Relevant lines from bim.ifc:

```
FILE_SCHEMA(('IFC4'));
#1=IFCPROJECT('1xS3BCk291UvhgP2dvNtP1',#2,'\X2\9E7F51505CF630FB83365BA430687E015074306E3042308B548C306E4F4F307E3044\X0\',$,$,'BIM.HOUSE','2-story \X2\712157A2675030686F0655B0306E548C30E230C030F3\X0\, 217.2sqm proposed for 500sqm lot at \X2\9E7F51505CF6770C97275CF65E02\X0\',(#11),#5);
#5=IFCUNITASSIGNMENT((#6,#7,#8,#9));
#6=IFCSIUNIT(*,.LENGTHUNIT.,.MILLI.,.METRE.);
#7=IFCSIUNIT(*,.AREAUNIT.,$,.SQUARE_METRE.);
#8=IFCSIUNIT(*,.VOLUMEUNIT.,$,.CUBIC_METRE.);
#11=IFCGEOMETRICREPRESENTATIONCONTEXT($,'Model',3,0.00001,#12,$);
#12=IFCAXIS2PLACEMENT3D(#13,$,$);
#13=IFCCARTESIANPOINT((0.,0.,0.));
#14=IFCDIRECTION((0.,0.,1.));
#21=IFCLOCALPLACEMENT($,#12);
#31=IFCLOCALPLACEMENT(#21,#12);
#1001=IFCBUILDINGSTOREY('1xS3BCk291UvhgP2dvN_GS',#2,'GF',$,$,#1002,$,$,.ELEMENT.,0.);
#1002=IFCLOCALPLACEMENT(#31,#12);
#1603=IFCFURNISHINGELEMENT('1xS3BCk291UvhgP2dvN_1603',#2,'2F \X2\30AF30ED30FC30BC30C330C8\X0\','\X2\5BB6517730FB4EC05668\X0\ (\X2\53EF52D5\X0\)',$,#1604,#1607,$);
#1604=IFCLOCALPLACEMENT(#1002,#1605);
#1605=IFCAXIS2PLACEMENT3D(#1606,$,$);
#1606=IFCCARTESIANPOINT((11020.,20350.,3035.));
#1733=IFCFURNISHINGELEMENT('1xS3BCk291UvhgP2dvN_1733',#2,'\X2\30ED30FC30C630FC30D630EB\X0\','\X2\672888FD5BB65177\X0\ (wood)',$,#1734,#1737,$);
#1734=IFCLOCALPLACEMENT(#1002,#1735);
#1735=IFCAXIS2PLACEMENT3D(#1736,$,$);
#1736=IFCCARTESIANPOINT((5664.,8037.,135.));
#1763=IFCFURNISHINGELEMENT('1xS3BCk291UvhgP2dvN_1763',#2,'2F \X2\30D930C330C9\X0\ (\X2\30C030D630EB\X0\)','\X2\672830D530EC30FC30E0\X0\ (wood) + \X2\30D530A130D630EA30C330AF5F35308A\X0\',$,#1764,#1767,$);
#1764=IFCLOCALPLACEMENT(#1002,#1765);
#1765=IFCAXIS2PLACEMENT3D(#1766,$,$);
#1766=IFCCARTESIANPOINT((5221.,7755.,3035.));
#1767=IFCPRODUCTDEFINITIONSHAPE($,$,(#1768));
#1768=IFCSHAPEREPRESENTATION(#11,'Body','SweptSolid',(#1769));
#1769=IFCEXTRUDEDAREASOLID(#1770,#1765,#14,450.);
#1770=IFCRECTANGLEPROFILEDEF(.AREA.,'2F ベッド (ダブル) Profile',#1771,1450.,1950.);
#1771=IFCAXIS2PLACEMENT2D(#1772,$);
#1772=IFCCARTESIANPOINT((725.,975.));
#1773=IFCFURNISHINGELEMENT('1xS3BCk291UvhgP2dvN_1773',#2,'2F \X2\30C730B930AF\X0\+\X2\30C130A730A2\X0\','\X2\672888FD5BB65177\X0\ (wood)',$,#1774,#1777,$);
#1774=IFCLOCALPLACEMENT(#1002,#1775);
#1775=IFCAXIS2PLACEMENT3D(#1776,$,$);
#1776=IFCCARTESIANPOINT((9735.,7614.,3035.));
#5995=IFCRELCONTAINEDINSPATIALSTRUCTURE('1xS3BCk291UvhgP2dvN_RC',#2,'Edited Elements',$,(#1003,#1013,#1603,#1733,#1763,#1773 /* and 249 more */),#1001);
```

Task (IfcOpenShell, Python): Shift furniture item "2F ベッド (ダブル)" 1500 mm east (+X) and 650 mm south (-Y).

```python
import ifcopenshell
import ifcopenshell.api.geometry
import ifcopenshell.util.placement

model = ifcopenshell.open("bim.ifc")

item = model.by_guid("1xS3BCk291UvhgP2dvN_1763")
matrix = ifcopenshell.util.placement.get_local_placement(item.ObjectPlacement)
matrix[0, 3] += 1500.0
matrix[1, 3] -= 650.0
ifcopenshell.api.geometry.edit_object_placement(model, product=item, matrix=matrix, is_si=False)

print(ifcopenshell.util.placement.get_local_placement(item.ObjectPlacement).round(3) + 0.0)

model.write("bim-out.ifc")
```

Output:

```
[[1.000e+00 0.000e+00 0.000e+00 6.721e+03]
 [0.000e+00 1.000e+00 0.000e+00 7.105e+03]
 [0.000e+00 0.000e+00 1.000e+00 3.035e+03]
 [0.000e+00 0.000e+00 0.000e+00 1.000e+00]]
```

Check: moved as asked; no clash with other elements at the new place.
